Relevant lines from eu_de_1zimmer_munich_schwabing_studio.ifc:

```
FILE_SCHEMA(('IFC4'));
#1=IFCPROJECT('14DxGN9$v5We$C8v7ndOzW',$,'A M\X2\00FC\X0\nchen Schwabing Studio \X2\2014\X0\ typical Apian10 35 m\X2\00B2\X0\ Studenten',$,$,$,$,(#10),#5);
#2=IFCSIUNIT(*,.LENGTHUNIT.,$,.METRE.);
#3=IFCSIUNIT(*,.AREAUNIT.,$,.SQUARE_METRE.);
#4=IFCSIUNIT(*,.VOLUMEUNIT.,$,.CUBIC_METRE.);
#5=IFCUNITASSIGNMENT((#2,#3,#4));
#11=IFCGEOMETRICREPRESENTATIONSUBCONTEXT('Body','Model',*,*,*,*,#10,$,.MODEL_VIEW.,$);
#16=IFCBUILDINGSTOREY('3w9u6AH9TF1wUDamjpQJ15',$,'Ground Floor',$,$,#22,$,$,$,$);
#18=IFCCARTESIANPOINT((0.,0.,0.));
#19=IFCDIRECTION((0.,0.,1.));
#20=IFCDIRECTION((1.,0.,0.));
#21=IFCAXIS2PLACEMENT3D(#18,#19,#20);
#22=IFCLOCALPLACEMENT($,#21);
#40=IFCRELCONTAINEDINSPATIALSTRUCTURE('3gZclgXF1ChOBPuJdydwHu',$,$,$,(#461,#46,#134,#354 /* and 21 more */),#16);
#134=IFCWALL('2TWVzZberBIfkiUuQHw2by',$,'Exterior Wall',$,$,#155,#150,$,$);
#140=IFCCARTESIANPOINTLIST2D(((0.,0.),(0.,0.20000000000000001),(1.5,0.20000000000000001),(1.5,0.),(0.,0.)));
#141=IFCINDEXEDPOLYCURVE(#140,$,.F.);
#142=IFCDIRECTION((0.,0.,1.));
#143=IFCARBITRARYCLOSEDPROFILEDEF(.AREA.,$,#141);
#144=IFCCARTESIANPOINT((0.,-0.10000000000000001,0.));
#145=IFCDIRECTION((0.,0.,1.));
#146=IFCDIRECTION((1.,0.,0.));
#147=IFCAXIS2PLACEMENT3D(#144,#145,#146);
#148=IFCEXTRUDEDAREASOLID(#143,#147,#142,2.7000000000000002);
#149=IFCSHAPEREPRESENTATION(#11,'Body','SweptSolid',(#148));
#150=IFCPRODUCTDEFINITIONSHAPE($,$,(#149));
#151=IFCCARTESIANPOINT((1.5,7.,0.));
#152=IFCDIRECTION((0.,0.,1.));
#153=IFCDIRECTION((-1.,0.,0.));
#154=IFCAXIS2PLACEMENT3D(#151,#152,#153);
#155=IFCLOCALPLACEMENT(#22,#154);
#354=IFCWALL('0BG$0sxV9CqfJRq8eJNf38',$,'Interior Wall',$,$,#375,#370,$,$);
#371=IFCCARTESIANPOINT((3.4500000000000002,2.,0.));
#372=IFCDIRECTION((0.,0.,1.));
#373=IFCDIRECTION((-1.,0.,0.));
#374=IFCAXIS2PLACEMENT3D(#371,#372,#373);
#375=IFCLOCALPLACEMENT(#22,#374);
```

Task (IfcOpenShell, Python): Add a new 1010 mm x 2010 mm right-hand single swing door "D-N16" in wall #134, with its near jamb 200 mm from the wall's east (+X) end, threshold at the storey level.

```python
import numpy as np
import ifcopenshell
import ifcopenshell.api.feature
import ifcopenshell.api.geometry
import ifcopenshell.api.root
import ifcopenshell.api.spatial
import ifcopenshell.geom
import ifcopenshell.util.element
import ifcopenshell.util.placement
import ifcopenshell.util.representation
import ifcopenshell.util.shape
import ifcopenshell.util.unit

model = ifcopenshell.open("eu_de_1zimmer_munich_schwabing_studio.ifc")
unit_scale = ifcopenshell.util.unit.calculate_unit_scale(model)
settings = ifcopenshell.geom.settings()


def volume(element):
    """Net volume in cubic metres, openings subtracted."""
    shape = ifcopenshell.geom.create_shape(settings, element)
    return ifcopenshell.util.shape.get_volume(shape.geometry)


wall = model.by_guid("2TWVzZberBIfkiUuQHw2by")
storey = ifcopenshell.util.element.get_container(wall, ifc_class="IfcBuildingStorey")
context = ifcopenshell.util.representation.get_context(model, "Model", "Body", "MODEL_VIEW")
before = volume(wall)

width, height, from_end, sill = 1.01, 2.01, 0.2, 0.0  # metres

# The wall runs along its own X axis, and the end named is its -X end.
wall_shape = ifcopenshell.geom.create_shape(settings, wall)
x, y, z = ifcopenshell.util.shape.get_vertices(wall_shape.geometry).T
start = x.min() + from_end
face, thickness = float(y.min()), float(y.max() - y.min())
wall_matrix = ifcopenshell.util.placement.get_local_placement(wall.ObjectPlacement)
level = ifcopenshell.util.placement.get_local_placement(storey.ObjectPlacement)[2, 3]


def in_wall(x, y):
    """Placement at x, y metres in the wall's axes, at sill height."""
    matrix = wall_matrix.copy()
    matrix[:, 3] = wall_matrix @ np.array([x / unit_scale, y / unit_scale, 0.0, 1.0])
    matrix[2, 3] = level + sill / unit_scale
    return matrix


# Opening: a box that overshoots both wall faces by 50 mm.
opening = ifcopenshell.api.root.create_entity(model, ifc_class="IfcOpeningElement", predefined_type="OPENING")
box = ifcopenshell.api.geometry.add_wall_representation(
    model, context=context, length=width, height=height, thickness=thickness + 0.1
)
ifcopenshell.api.geometry.assign_representation(model, product=opening, representation=box)
ifcopenshell.api.geometry.edit_object_placement(model, product=opening, matrix=in_wall(start, face - 0.05), is_si=False)
ifcopenshell.api.feature.add_feature(model, feature=opening, element=wall)

door = ifcopenshell.api.root.create_entity(model, ifc_class="IfcDoor", name="D-N16", predefined_type="DOOR")
door.OverallWidth, door.OverallHeight = width / unit_scale, height / unit_scale
door.OperationType = "SINGLE_SWING_RIGHT"
body = ifcopenshell.api.geometry.add_door_representation(
    model,
    context=context,
    overall_width=door.OverallWidth,
    overall_height=door.OverallHeight,
    operation_type="SINGLE_SWING_RIGHT",
    lining_properties={"LiningDepth": thickness / unit_scale, "ThresholdDepth": thickness / unit_scale},
)
ifcopenshell.api.geometry.assign_representation(model, product=door, representation=body)
ifcopenshell.api.spatial.assign_container(model, products=[door], relating_structure=storey)
ifcopenshell.api.feature.add_filling(model, opening=opening, element=door)

# The lining spans the wall, so the door starts at the wall face.
ifcopenshell.api.geometry.edit_object_placement(model, product=door, matrix=in_wall(start, face), is_si=False)

after = volume(wall)

print(f"wall volume {before:.3f} -> {after:.3f} m3")

model.write("eu_de_1zimmer_munich_schwabing_studio-out.ifc")
```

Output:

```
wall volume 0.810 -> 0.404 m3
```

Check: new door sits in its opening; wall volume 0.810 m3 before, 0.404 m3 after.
